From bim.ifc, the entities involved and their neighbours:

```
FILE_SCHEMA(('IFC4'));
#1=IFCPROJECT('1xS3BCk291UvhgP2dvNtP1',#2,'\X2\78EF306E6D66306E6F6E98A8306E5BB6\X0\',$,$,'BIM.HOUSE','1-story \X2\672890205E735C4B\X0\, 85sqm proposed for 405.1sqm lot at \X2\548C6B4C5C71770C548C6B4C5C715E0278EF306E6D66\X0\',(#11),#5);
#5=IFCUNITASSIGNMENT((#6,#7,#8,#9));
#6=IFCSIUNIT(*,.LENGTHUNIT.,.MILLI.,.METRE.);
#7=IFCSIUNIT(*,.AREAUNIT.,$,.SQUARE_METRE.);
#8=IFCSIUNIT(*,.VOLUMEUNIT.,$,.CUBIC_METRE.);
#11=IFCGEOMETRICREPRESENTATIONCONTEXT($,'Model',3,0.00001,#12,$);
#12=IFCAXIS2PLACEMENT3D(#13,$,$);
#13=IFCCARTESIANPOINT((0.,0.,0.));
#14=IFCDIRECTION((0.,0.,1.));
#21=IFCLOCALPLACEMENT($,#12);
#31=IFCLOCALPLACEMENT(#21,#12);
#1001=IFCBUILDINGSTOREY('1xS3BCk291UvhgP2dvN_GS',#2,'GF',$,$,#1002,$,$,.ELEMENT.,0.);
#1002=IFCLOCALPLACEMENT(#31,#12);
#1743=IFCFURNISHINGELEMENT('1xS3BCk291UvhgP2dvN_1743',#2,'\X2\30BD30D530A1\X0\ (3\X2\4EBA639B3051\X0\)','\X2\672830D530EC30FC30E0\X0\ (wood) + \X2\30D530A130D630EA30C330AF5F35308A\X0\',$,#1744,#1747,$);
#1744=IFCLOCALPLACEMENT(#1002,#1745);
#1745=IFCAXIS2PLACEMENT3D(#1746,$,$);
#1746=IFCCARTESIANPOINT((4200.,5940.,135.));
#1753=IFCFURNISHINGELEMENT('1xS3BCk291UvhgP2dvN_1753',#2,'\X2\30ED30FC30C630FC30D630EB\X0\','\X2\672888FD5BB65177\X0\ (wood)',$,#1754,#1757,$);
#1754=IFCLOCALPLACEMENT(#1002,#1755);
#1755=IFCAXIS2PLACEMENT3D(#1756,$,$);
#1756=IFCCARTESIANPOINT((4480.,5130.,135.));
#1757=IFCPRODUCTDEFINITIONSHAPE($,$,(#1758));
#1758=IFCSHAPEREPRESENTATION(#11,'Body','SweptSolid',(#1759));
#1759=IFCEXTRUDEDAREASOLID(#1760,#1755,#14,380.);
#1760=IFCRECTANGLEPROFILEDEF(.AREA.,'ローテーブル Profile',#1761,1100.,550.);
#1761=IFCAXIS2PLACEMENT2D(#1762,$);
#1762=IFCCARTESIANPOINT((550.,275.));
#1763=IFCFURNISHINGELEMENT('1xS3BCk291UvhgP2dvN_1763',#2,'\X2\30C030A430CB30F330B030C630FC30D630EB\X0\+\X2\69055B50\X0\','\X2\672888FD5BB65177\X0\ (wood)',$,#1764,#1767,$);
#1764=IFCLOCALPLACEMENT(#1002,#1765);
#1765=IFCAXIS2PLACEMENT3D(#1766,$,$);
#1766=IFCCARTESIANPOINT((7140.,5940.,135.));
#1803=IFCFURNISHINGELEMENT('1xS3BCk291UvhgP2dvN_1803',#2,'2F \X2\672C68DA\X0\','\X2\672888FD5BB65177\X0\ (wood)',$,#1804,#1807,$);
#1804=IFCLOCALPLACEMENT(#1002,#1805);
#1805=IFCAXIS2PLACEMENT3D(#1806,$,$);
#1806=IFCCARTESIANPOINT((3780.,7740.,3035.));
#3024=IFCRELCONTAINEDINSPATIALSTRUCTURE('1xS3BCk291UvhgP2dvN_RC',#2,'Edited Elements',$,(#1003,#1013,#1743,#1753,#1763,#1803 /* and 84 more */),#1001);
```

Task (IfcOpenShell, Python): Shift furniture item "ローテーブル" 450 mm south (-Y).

```python
import ifcopenshell
import ifcopenshell.api.geometry
import ifcopenshell.util.placement

model = ifcopenshell.open("bim.ifc")

item = model.by_guid("1xS3BCk291UvhgP2dvN_1753")
matrix = ifcopenshell.util.placement.get_local_placement(item.ObjectPlacement)
matrix[1, 3] -= 450.0
ifcopenshell.api.geometry.edit_object_placement(model, product=item, matrix=matrix, is_si=False)

print(ifcopenshell.util.placement.get_local_placement(item.ObjectPlacement).round(3) + 0.0)

model.write("bim_v2.ifc")
```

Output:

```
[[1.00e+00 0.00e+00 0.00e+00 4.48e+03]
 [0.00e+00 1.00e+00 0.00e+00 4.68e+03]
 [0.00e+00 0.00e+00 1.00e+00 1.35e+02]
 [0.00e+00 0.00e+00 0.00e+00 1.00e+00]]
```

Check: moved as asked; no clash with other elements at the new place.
